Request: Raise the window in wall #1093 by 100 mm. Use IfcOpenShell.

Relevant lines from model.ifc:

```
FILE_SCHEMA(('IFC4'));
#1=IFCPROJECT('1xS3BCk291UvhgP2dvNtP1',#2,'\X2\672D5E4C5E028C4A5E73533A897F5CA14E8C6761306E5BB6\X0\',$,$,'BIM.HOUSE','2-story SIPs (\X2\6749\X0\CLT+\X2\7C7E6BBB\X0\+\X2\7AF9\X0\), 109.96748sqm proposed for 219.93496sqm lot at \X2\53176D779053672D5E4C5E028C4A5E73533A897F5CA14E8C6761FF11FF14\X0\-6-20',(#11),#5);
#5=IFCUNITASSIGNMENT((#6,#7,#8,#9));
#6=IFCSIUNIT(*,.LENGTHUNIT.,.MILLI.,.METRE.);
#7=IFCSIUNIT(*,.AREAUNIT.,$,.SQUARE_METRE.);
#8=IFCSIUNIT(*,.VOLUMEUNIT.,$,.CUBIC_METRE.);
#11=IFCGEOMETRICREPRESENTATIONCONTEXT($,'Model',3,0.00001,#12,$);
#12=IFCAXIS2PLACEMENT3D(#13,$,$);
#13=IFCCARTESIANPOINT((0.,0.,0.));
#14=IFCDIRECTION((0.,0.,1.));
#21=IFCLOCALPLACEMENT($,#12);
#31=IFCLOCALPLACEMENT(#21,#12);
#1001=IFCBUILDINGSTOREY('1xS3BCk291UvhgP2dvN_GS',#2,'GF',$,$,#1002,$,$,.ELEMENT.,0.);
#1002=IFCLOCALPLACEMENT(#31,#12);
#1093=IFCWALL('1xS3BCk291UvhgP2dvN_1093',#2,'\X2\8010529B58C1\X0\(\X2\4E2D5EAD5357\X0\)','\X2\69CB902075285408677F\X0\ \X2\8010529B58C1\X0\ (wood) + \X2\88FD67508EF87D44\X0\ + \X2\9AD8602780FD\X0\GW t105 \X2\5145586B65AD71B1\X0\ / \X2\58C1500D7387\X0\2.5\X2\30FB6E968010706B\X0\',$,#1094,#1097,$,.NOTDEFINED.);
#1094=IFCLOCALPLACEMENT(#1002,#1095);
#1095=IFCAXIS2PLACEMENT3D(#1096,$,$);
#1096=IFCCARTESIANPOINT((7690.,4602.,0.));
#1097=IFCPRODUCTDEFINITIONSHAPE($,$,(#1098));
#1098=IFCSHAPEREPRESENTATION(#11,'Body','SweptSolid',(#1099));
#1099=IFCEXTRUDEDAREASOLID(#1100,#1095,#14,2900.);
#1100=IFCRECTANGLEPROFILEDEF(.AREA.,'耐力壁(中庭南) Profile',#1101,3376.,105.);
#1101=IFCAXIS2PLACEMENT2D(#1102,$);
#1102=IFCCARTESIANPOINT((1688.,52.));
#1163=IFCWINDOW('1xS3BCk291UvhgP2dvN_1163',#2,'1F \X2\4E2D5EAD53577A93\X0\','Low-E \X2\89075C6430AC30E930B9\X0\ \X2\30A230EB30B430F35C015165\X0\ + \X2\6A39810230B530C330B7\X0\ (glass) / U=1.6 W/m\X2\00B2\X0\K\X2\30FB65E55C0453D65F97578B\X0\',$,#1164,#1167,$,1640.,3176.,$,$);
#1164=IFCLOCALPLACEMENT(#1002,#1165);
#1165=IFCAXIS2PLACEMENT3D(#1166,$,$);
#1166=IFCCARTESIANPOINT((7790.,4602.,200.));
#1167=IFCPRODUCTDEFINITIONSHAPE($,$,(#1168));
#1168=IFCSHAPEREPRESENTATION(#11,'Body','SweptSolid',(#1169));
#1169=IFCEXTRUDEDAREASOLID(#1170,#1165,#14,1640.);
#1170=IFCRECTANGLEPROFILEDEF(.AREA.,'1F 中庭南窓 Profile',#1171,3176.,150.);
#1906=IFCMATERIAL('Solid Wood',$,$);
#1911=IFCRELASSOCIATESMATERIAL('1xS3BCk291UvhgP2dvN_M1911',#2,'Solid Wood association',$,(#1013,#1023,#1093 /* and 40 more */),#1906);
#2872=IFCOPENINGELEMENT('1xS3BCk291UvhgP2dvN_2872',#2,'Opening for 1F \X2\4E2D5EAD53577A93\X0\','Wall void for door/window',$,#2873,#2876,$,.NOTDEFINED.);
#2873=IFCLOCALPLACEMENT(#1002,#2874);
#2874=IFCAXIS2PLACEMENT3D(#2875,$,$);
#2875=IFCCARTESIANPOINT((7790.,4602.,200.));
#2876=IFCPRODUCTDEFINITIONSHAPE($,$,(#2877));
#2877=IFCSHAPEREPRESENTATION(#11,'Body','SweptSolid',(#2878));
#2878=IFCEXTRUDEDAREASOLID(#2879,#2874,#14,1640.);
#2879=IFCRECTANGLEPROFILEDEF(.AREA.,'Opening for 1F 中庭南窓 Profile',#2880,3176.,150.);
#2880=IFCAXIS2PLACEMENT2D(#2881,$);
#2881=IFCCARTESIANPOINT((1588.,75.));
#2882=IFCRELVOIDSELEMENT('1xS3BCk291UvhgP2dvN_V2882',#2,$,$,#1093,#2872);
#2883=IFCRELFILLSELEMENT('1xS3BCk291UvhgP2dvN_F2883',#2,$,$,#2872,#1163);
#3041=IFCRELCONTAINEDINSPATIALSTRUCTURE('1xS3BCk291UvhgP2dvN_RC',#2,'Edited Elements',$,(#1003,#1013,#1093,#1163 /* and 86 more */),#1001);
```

```python
import numpy as np
import ifcopenshell
import ifcopenshell.api.geometry
import ifcopenshell.util.placement
import ifcopenshell.util.unit

model = ifcopenshell.open("model.ifc")
unit_scale = ifcopenshell.util.unit.calculate_unit_scale(model)

window = model.by_guid("1xS3BCk291UvhgP2dvN_1163")
opening = window.FillsVoids[0].RelatingOpeningElement
dz = 0.1 / unit_scale

shift = np.array([0.0, 0.0, dz])
# The window is not placed relative to its opening, so move both.
for product in (opening, window):
    matrix = ifcopenshell.util.placement.get_local_placement(product.ObjectPlacement)
    matrix[:3, 3] += shift
    ifcopenshell.api.geometry.edit_object_placement(model, product=product, matrix=matrix, is_si=False)

print(f"moved by {dz * unit_scale:+.3f} m")

model.write("model_v2.ifc")
```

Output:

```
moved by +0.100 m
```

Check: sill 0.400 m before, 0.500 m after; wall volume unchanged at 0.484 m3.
